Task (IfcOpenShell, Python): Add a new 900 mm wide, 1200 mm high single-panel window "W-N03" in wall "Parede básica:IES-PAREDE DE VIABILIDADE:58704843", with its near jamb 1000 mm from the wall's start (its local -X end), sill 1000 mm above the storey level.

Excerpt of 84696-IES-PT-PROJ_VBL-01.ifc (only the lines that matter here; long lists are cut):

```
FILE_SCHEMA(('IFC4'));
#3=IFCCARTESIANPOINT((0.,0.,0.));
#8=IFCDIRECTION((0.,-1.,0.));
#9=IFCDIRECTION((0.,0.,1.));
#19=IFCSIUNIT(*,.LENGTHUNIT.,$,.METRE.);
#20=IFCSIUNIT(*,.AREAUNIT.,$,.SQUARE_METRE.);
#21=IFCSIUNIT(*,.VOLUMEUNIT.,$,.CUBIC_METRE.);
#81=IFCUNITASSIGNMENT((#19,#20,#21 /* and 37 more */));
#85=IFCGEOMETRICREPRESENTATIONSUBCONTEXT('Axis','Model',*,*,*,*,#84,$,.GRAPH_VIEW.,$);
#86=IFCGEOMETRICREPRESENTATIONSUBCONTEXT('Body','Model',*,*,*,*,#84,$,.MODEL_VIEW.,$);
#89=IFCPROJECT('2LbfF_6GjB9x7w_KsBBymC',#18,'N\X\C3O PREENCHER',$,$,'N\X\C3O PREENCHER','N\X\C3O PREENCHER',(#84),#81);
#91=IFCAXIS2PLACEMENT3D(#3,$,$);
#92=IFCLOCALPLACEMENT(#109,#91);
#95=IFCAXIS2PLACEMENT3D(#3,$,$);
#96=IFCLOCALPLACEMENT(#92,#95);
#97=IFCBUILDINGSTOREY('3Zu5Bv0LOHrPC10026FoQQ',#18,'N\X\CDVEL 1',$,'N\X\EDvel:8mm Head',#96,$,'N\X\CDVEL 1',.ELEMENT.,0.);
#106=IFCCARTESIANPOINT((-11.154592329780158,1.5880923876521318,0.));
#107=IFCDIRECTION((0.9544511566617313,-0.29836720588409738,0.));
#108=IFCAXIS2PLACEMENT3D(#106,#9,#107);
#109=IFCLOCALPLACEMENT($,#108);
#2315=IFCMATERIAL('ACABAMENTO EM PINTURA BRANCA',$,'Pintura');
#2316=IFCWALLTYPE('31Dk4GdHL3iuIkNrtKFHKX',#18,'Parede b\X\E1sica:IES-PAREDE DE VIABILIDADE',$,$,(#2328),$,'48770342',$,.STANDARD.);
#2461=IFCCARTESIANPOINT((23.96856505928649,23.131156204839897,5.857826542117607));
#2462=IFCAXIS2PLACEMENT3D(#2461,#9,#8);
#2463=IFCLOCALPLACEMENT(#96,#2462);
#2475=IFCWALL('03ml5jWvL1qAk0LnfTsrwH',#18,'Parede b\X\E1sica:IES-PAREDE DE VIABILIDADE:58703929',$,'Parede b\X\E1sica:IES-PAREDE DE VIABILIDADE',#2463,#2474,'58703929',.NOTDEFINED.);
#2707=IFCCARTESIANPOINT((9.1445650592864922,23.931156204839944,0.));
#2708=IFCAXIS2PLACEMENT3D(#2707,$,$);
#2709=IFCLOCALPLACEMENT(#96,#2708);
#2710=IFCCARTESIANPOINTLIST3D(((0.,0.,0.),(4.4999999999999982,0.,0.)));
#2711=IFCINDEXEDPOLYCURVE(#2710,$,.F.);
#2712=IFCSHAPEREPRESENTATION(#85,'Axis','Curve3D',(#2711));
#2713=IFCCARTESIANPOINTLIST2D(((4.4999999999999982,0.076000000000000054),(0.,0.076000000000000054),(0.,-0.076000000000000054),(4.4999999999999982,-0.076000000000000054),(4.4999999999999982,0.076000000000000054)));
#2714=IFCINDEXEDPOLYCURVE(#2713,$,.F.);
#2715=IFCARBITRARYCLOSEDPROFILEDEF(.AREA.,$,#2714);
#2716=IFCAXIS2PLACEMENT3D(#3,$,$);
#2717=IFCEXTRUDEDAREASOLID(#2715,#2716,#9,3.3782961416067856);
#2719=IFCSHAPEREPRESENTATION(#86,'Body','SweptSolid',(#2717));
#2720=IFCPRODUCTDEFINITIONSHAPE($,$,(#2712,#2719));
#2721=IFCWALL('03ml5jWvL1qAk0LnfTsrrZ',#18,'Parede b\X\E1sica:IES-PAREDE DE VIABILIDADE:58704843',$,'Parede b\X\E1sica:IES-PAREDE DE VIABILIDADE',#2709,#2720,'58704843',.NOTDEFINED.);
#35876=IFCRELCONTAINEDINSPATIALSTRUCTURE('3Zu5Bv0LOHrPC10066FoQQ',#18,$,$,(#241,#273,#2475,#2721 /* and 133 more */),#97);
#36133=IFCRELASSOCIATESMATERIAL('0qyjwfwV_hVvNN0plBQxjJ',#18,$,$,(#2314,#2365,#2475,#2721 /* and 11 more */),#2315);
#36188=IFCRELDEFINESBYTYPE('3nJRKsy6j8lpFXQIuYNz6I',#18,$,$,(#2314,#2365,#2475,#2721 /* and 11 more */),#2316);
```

```python
import numpy as np
import ifcopenshell
import ifcopenshell.api.feature
import ifcopenshell.api.geometry
import ifcopenshell.api.root
import ifcopenshell.api.spatial
import ifcopenshell.geom
import ifcopenshell.util.element
import ifcopenshell.util.placement
import ifcopenshell.util.representation
import ifcopenshell.util.shape
import ifcopenshell.util.unit

model = ifcopenshell.open("84696-IES-PT-PROJ_VBL-01.ifc")
unit_scale = ifcopenshell.util.unit.calculate_unit_scale(model)
settings = ifcopenshell.geom.settings()


def volume(element):
    """Net volume in cubic metres, openings subtracted."""
    shape = ifcopenshell.geom.create_shape(settings, element)
    return ifcopenshell.util.shape.get_volume(shape.geometry)


wall = model.by_guid("03ml5jWvL1qAk0LnfTsrrZ")
storey = ifcopenshell.util.element.get_container(wall, ifc_class="IfcBuildingStorey")
context = ifcopenshell.util.representation.get_context(model, "Model", "Body", "MODEL_VIEW")
before = volume(wall)

width, height, from_end, sill = 0.9, 1.2, 1, 1  # metres

# The wall runs along its own X axis, and the end named is its -X end.
wall_shape = ifcopenshell.geom.create_shape(settings, wall)
x, y, z = ifcopenshell.util.shape.get_vertices(wall_shape.geometry).T
start = x.min() + from_end
face, thickness = float(y.min()), float(y.max() - y.min())
wall_matrix = ifcopenshell.util.placement.get_local_placement(wall.ObjectPlacement)
level = ifcopenshell.util.placement.get_local_placement(storey.ObjectPlacement)[2, 3]


def in_wall(x, y):
    """Placement at x, y metres in the wall's axes, at sill height."""
    matrix = wall_matrix.copy()
    matrix[:, 3] = wall_matrix @ np.array([x / unit_scale, y / unit_scale, 0.0, 1.0])
    matrix[2, 3] = level + sill / unit_scale
    return matrix


# Opening: a box that overshoots both wall faces by 50 mm.
opening = ifcopenshell.api.root.create_entity(model, ifc_class="IfcOpeningElement", predefined_type="OPENING")
box = ifcopenshell.api.geometry.add_wall_representation(
    model, context=context, length=width, height=height, thickness=thickness + 0.1
)
ifcopenshell.api.geometry.assign_representation(model, product=opening, representation=box)
ifcopenshell.api.geometry.edit_object_placement(model, product=opening, matrix=in_wall(start, face - 0.05), is_si=False)
ifcopenshell.api.feature.add_feature(model, feature=opening, element=wall)

window = ifcopenshell.api.root.create_entity(model, ifc_class="IfcWindow", name="W-N03", predefined_type="WINDOW")
window.OverallWidth, window.OverallHeight = width / unit_scale, height / unit_scale
window.PartitioningType = "SINGLE_PANEL"
body = ifcopenshell.api.geometry.add_window_representation(
    model,
    context=context,
    overall_width=window.OverallWidth,
    overall_height=window.OverallHeight,
    partition_type="SINGLE_PANEL",
)
ifcopenshell.api.geometry.assign_representation(model, product=window, representation=body)
ifcopenshell.api.spatial.assign_container(model, products=[window], relating_structure=storey)
ifcopenshell.api.feature.add_filling(model, opening=opening, element=window)

# Centre the window in the wall's thickness.
ifcopenshell.api.geometry.edit_object_placement(model, product=window, matrix=in_wall(start, face), is_si=False)
window_shape = ifcopenshell.geom.create_shape(settings, window)
depth = ifcopenshell.util.shape.get_vertices(window_shape.geometry)[:, 1]
offset = face + thickness / 2 - (depth.min() + depth.max()) / 2
ifcopenshell.api.geometry.edit_object_placement(model, product=window, matrix=in_wall(start, offset), is_si=False)

after = volume(wall)

print(f"wall volume {before:.3f} -> {after:.3f} m3")

model.write("84696-IES-PT-PROJ_VBL-01_updated.ifc")
```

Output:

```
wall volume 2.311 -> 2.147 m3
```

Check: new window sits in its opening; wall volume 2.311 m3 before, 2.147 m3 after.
